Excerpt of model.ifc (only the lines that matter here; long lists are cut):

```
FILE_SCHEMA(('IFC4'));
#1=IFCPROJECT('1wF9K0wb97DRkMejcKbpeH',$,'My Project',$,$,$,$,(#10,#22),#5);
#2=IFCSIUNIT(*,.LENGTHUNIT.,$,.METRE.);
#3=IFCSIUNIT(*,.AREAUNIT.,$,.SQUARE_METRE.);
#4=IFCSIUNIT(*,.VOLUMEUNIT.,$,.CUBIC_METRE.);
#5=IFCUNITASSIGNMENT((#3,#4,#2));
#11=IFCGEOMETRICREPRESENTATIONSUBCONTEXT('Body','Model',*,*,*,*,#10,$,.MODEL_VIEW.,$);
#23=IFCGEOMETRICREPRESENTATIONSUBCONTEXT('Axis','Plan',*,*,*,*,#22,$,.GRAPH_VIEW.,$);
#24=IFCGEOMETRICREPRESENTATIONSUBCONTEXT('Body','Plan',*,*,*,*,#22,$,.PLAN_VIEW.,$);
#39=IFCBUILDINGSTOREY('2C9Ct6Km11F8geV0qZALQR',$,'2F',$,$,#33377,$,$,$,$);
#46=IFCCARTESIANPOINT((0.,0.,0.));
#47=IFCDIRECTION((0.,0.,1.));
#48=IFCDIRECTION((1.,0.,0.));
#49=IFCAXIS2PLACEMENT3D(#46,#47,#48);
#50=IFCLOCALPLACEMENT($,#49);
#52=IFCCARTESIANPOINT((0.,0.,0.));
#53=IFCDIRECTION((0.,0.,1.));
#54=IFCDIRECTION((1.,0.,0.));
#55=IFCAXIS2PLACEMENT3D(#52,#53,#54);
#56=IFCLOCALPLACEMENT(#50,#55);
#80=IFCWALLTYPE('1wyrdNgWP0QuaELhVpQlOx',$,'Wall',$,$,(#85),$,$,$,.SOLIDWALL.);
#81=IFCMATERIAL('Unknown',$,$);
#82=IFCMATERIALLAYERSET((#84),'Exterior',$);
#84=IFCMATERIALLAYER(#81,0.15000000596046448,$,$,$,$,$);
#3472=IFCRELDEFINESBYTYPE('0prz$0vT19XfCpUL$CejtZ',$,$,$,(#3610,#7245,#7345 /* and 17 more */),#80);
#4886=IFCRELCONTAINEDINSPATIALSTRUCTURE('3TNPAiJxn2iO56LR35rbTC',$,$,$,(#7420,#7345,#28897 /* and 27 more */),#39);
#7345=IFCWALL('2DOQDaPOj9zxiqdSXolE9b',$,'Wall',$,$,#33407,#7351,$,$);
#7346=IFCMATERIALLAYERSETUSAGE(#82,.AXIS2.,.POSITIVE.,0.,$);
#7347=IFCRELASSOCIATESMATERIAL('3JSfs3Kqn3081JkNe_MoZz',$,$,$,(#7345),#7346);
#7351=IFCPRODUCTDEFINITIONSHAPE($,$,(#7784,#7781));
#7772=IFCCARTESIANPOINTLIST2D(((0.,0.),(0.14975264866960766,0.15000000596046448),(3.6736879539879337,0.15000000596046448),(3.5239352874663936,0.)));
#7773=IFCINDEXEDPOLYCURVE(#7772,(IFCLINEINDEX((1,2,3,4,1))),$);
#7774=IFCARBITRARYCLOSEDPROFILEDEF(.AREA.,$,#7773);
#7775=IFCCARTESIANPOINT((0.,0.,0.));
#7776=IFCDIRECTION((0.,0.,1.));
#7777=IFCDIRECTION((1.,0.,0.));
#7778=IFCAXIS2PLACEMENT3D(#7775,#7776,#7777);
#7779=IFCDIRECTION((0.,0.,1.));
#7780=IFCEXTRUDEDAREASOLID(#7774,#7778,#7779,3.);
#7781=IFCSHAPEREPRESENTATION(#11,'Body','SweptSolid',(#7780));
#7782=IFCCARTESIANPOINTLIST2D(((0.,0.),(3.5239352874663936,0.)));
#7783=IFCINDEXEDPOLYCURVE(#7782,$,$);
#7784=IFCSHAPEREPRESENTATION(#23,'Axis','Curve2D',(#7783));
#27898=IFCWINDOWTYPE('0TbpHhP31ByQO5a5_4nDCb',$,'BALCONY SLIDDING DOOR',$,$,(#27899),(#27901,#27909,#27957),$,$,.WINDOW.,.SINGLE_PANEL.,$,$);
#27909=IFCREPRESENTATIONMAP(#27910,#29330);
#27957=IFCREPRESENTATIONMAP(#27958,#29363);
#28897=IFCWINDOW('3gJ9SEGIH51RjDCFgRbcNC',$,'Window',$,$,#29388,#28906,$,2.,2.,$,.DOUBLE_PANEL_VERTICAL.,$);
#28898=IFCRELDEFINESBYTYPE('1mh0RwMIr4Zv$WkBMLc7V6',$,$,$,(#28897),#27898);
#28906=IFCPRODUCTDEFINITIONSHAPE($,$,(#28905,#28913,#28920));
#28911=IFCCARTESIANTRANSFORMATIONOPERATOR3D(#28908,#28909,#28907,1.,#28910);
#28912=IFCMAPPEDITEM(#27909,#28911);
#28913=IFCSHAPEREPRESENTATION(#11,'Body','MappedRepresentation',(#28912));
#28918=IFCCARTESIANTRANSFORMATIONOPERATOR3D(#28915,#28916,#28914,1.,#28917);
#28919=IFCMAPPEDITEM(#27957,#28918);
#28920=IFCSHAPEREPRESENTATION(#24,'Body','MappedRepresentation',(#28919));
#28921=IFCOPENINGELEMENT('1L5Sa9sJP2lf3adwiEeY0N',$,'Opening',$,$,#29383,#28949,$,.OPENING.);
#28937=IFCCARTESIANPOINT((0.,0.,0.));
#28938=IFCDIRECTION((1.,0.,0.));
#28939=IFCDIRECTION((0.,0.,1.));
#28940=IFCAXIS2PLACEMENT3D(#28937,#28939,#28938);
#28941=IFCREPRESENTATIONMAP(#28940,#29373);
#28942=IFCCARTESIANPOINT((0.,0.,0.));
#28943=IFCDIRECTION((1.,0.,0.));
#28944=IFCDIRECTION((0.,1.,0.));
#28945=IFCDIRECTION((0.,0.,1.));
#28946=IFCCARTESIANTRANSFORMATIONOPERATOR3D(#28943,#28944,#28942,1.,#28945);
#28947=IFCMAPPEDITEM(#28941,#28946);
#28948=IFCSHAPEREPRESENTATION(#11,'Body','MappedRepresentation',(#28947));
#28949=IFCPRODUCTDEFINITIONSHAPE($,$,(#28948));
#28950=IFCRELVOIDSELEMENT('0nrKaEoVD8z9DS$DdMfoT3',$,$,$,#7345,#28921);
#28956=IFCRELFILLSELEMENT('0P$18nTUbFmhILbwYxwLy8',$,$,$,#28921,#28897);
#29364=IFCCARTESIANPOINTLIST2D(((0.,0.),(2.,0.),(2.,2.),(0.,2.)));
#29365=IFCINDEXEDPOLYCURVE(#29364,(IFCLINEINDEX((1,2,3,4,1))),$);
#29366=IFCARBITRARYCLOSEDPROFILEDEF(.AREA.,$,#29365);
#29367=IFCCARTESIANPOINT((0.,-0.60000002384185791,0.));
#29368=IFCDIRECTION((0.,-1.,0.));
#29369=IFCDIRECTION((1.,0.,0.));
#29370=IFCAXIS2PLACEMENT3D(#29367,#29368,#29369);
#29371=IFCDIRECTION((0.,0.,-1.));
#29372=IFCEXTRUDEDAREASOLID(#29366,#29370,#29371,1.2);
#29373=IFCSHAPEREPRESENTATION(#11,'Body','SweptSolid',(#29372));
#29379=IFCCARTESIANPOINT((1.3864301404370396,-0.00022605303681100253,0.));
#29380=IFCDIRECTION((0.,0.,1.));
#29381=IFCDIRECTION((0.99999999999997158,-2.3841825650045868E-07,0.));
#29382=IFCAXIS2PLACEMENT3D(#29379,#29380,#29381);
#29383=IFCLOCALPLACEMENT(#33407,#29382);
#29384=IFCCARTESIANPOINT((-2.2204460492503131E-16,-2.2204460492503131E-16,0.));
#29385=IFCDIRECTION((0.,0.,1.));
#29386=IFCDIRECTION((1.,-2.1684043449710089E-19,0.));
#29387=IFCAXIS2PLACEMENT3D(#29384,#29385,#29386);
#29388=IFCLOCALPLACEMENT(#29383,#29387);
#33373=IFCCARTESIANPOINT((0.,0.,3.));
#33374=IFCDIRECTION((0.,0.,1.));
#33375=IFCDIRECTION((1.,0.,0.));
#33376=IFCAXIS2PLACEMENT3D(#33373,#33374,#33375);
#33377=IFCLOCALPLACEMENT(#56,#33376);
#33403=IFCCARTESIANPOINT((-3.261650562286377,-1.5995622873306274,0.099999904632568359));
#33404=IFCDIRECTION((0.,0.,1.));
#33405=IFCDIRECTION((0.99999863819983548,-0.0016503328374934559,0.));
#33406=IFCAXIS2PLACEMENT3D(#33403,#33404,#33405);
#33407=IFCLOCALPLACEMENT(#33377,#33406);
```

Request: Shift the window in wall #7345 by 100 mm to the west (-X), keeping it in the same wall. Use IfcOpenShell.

```python
import ifcopenshell
import ifcopenshell.api.geometry
import ifcopenshell.util.placement

model = ifcopenshell.open("model.ifc")

window = model.by_guid("3gJ9SEGIH51RjDCFgRbcNC")
opening = window.FillsVoids[0].RelatingOpeningElement
wall = opening.VoidsElements[0].RelatingBuildingElement

wall_matrix = ifcopenshell.util.placement.get_local_placement(wall.ObjectPlacement)
shift = wall_matrix[:3, 0] * -0.1
before = ifcopenshell.util.placement.get_local_placement(window.ObjectPlacement)[:3, 3].copy()

# The window is placed relative to its opening, so it follows when the opening moves.
matrix = ifcopenshell.util.placement.get_local_placement(opening.ObjectPlacement)
matrix[:3, 3] += shift
ifcopenshell.api.geometry.edit_object_placement(
    model, product=opening, matrix=matrix, is_si=False, should_transform_children=True
)

after = ifcopenshell.util.placement.get_local_placement(window.ObjectPlacement)[:3, 3]
print("window moved by", (after - before).round(3) + 0.0)

model.write("model_edited.ifc")
```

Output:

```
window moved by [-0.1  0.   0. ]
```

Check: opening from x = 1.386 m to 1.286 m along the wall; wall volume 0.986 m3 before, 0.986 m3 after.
